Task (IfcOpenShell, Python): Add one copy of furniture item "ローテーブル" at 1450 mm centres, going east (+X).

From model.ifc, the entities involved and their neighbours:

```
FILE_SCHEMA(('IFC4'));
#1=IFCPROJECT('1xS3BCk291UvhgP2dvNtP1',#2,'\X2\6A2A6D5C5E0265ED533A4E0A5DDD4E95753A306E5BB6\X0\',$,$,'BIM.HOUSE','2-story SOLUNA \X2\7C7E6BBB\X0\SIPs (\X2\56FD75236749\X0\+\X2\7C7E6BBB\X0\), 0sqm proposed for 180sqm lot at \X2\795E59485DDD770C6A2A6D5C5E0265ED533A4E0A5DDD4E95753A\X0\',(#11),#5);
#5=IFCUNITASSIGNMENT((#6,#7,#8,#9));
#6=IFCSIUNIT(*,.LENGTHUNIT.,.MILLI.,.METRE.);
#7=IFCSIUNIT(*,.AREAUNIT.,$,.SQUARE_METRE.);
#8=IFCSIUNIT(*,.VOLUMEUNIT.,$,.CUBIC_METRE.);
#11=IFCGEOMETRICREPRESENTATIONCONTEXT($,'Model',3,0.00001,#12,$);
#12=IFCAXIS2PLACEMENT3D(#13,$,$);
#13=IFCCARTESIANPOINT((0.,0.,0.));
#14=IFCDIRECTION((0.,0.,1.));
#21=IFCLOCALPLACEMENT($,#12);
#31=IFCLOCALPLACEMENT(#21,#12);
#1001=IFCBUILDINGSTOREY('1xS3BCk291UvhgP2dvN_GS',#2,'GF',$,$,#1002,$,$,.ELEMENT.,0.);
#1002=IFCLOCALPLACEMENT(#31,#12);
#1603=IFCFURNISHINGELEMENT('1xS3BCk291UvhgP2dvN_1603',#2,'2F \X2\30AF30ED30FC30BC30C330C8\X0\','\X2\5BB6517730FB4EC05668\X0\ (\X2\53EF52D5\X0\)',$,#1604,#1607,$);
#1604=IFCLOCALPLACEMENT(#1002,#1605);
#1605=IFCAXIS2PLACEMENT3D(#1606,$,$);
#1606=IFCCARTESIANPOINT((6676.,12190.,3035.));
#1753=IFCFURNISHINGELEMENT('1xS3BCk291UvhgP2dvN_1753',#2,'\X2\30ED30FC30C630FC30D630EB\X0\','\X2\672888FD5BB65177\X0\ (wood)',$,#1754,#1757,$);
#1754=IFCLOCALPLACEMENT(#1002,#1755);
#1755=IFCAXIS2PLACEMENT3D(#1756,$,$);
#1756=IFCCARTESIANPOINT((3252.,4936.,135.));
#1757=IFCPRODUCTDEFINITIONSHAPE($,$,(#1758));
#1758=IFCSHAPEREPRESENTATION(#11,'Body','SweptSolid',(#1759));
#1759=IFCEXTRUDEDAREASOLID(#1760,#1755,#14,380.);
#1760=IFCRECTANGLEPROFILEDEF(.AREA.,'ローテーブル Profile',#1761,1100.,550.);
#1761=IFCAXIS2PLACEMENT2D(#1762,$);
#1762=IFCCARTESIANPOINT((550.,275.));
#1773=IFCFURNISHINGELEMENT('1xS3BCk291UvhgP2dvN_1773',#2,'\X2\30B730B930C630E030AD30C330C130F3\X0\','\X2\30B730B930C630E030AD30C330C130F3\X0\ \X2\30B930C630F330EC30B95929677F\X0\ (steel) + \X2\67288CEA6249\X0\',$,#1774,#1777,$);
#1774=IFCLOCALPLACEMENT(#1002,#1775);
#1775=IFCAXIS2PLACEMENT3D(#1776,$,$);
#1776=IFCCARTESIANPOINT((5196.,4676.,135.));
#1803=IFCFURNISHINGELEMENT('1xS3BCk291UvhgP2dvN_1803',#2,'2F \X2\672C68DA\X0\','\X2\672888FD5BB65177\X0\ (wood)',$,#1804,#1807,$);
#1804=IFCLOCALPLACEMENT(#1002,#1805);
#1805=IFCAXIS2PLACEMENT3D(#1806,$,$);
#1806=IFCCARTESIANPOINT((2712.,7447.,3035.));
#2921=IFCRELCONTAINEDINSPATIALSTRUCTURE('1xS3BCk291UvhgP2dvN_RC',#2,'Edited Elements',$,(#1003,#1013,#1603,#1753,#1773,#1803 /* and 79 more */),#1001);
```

```python
import numpy as np
import ifcopenshell
import ifcopenshell.api.geometry
import ifcopenshell.api.root
import ifcopenshell.util.element
import ifcopenshell.util.placement
import ifcopenshell.util.unit

model = ifcopenshell.open("model.ifc")
unit_scale = ifcopenshell.util.unit.calculate_unit_scale(model)


def reuse_history(source, copy):
    """copy_class also copies each property set's owner history, people and application; keep the originals."""
    for rel in copy.IsDefinedBy:
        if rel.is_a("IfcRelDefinesByProperties") and (history := rel.RelatingPropertyDefinition.OwnerHistory):
            rel.RelatingPropertyDefinition.OwnerHistory = source.OwnerHistory
            ifcopenshell.util.element.remove_deep2(model, history)


source = model.by_guid("1xS3BCk291UvhgP2dvN_1753")
base = ifcopenshell.util.placement.get_local_placement(source.ObjectPlacement)
step = np.array([1.0, 0.0, 0.0]) * 1.45 / unit_scale

for i in range(1, 2):
    copy = ifcopenshell.api.root.copy_class(model, product=source)
    copy.Representation = ifcopenshell.util.element.copy_deep(
        model, source.Representation, exclude=["IfcGeometricRepresentationContext", "IfcRepresentationMap"]
    )
    reuse_history(source, copy)
    matrix = base.copy()
    matrix[:3, 3] += i * step
    print("added at", matrix[:3, 3].round(3) + 0.0)
    ifcopenshell.api.geometry.edit_object_placement(model, product=copy, matrix=matrix, is_si=False)

model.write("model_v2.ifc")
```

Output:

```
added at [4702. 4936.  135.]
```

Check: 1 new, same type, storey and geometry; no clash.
